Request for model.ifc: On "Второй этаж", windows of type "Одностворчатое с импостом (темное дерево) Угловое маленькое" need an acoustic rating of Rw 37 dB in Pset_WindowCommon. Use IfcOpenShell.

First a look at what the model holds.

```python
import ifcopenshell
import ifcopenshell.util.element

model = ifcopenshell.open("model.ifc")
print(model.schema)
storey = next(s for s in model.by_type("IfcBuildingStorey") if s.Name == "Второй этаж")
windows = [e for e in ifcopenshell.util.element.get_decomposition(storey) if e.is_a("IfcWindow")]
seen = {}
for e in windows:
    element_type = ifcopenshell.util.element.get_type(e)
    key = (element_type.Name if element_type != e and element_type else None, ifcopenshell.util.element.get_pset(e, "Pset_WindowCommon", "AcousticRating"))
    seen[key] = seen.get(key, 0) + 1
for (name, value), count in sorted(seen.items(), key=str):
    print(count, "x", name, "|", value)
```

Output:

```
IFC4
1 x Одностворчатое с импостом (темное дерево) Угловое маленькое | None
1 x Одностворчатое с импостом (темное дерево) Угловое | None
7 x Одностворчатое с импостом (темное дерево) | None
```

```python
import ifcopenshell
import ifcopenshell.api.pset
import ifcopenshell.util.element

model = ifcopenshell.open("model.ifc")

storey = next(s for s in model.by_type("IfcBuildingStorey") if s.Name == "Второй этаж")
windows = [e for e in ifcopenshell.util.element.get_decomposition(storey) if e.is_a("IfcWindow")]

count = 0
for e in windows:
    element_type = ifcopenshell.util.element.get_type(e)
    if element_type in (None, e) or element_type.Name != "Одностворчатое с импостом (темное дерево) Угловое маленькое":
        continue
    # add_pset returns the element's existing set when there is one.
    pset = ifcopenshell.api.pset.add_pset(model, product=e, name="Pset_WindowCommon")
    ifcopenshell.api.pset.edit_pset(model, pset=pset, properties={"AcousticRating": "Rw 37 dB"})
    count += 1

print(count, "windows updated")

model.write("model_edited.ifc")
```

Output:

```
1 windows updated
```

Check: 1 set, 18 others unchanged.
